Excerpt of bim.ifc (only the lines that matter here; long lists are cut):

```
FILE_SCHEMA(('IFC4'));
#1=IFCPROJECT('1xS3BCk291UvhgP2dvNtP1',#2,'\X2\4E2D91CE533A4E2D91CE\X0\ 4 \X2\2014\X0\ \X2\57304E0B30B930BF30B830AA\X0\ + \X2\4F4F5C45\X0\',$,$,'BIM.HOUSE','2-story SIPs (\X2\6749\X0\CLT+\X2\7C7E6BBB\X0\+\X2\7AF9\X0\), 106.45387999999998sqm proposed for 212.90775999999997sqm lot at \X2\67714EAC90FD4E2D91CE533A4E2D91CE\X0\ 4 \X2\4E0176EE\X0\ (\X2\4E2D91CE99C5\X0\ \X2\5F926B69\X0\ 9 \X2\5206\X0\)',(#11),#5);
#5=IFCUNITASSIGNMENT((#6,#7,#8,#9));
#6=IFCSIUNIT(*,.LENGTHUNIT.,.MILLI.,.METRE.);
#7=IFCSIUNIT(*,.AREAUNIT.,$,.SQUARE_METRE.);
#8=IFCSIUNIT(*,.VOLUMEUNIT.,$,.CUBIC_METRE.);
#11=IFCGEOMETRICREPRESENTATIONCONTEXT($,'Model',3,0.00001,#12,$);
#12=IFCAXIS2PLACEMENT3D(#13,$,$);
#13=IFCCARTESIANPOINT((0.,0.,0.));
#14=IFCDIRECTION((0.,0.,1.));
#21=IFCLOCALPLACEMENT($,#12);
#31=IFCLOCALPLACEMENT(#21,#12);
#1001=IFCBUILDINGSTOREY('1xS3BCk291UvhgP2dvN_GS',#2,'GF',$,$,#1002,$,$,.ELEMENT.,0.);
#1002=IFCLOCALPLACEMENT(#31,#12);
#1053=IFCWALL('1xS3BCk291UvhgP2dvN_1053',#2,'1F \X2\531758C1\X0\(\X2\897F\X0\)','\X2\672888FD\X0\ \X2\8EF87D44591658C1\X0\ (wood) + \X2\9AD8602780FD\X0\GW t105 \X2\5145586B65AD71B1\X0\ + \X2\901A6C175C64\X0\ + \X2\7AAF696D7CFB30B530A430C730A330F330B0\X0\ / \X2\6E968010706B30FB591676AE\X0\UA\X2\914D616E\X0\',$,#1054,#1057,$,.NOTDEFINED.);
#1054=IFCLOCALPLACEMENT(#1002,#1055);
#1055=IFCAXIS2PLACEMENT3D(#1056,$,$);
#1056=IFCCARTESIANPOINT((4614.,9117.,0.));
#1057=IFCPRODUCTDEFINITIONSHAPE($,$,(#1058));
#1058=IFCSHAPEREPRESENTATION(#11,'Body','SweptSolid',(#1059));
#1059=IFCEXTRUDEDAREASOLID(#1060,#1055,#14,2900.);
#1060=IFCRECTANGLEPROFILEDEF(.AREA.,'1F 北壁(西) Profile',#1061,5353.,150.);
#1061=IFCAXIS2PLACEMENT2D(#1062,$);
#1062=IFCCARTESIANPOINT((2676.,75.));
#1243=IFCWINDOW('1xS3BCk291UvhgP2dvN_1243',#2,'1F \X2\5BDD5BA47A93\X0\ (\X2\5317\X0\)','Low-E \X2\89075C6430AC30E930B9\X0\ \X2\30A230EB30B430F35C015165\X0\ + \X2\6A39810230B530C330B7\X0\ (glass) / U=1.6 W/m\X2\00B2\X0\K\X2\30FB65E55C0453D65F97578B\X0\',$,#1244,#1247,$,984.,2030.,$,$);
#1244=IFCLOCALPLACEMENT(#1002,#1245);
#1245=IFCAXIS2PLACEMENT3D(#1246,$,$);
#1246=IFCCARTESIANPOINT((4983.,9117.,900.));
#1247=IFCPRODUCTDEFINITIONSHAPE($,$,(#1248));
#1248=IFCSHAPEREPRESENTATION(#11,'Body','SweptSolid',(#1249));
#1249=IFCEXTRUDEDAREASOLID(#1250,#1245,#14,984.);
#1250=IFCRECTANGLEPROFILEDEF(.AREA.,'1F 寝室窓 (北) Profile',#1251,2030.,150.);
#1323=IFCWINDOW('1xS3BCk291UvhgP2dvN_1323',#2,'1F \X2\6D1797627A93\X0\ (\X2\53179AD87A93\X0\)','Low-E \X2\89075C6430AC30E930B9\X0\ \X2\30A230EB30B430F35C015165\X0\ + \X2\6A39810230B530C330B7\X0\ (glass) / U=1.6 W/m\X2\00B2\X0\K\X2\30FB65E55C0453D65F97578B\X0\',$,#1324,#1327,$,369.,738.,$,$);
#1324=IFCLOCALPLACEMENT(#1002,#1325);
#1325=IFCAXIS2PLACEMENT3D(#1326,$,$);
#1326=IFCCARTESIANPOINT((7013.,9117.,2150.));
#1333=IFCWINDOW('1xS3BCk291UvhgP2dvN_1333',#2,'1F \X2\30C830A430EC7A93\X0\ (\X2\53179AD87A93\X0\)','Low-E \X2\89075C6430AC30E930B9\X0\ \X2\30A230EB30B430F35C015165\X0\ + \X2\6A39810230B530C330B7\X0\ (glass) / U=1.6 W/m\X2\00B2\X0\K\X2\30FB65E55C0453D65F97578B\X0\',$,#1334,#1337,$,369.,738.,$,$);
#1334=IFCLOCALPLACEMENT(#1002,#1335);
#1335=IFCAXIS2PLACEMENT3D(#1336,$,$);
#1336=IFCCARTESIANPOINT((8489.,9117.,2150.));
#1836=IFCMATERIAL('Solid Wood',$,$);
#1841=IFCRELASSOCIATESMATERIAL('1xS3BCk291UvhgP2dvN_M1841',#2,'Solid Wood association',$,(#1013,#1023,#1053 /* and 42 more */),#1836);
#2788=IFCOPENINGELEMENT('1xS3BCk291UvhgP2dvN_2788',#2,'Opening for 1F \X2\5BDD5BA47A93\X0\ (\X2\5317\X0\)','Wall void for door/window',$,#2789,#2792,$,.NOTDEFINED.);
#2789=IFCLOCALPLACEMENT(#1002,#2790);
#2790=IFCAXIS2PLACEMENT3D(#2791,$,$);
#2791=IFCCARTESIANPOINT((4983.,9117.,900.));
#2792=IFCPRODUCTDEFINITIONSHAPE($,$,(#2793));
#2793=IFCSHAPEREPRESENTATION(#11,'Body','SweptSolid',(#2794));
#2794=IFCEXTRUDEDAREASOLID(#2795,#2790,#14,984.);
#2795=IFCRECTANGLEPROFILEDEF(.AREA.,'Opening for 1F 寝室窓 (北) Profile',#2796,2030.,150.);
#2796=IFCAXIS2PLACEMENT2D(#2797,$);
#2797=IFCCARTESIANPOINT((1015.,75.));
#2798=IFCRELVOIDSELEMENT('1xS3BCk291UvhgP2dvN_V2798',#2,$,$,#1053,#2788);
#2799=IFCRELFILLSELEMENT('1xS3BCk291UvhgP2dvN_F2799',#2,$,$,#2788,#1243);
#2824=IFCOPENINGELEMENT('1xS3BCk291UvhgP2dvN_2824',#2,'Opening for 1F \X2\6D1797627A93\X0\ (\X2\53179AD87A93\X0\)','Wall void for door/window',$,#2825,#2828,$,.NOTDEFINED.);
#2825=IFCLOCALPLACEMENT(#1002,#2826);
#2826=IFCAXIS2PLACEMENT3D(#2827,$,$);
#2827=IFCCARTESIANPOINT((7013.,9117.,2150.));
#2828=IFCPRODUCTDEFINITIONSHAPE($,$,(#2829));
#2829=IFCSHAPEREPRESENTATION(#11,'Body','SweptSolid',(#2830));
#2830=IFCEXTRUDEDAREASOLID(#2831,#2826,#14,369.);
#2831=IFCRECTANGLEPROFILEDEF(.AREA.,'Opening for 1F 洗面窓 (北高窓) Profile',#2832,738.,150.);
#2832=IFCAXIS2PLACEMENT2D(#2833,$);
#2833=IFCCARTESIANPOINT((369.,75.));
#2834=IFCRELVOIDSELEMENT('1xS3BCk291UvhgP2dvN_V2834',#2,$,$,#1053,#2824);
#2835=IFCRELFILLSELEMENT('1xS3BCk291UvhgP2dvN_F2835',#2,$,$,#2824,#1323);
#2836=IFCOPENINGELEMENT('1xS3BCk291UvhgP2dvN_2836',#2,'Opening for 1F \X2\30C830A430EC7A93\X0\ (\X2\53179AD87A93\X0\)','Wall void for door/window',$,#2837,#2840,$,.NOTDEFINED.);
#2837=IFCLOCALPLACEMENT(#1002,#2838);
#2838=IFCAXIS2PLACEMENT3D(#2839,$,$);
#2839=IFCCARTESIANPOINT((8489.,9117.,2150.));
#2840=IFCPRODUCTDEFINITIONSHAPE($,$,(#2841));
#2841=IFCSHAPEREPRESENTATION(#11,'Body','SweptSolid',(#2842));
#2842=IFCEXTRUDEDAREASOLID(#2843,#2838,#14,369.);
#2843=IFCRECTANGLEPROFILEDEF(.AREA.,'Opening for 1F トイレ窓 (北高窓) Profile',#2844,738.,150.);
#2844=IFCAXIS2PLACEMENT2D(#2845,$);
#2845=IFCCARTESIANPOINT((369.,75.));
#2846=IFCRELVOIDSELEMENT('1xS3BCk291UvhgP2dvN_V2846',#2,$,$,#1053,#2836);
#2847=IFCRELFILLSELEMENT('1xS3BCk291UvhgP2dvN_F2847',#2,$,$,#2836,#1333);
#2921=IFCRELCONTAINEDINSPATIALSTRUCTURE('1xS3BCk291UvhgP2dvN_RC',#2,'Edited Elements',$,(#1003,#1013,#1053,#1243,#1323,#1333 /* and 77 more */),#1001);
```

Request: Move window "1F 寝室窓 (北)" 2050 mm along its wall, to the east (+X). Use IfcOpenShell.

```python
import ifcopenshell
import ifcopenshell.api.geometry
import ifcopenshell.util.placement
import ifcopenshell.util.unit

model = ifcopenshell.open("bim.ifc")
unit_scale = ifcopenshell.util.unit.calculate_unit_scale(model)

window = model.by_guid("1xS3BCk291UvhgP2dvN_1243")
opening = window.FillsVoids[0].RelatingOpeningElement
wall = opening.VoidsElements[0].RelatingBuildingElement

wall_matrix = ifcopenshell.util.placement.get_local_placement(wall.ObjectPlacement)
shift = wall_matrix[:3, 0] * 2.05 / unit_scale
before = ifcopenshell.util.placement.get_local_placement(window.ObjectPlacement)[:3, 3].copy()

# The window is not placed relative to its opening, so move both.
for product in (opening, window):
    matrix = ifcopenshell.util.placement.get_local_placement(product.ObjectPlacement)
    matrix[:3, 3] += shift
    ifcopenshell.api.geometry.edit_object_placement(model, product=product, matrix=matrix, is_si=False)

after = ifcopenshell.util.placement.get_local_placement(window.ObjectPlacement)[:3, 3]
print("window moved by", (after - before).round(3) + 0.0)

model.write("bim_edited.ifc")
```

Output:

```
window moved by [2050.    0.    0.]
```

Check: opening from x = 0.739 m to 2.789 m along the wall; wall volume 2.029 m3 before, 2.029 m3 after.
